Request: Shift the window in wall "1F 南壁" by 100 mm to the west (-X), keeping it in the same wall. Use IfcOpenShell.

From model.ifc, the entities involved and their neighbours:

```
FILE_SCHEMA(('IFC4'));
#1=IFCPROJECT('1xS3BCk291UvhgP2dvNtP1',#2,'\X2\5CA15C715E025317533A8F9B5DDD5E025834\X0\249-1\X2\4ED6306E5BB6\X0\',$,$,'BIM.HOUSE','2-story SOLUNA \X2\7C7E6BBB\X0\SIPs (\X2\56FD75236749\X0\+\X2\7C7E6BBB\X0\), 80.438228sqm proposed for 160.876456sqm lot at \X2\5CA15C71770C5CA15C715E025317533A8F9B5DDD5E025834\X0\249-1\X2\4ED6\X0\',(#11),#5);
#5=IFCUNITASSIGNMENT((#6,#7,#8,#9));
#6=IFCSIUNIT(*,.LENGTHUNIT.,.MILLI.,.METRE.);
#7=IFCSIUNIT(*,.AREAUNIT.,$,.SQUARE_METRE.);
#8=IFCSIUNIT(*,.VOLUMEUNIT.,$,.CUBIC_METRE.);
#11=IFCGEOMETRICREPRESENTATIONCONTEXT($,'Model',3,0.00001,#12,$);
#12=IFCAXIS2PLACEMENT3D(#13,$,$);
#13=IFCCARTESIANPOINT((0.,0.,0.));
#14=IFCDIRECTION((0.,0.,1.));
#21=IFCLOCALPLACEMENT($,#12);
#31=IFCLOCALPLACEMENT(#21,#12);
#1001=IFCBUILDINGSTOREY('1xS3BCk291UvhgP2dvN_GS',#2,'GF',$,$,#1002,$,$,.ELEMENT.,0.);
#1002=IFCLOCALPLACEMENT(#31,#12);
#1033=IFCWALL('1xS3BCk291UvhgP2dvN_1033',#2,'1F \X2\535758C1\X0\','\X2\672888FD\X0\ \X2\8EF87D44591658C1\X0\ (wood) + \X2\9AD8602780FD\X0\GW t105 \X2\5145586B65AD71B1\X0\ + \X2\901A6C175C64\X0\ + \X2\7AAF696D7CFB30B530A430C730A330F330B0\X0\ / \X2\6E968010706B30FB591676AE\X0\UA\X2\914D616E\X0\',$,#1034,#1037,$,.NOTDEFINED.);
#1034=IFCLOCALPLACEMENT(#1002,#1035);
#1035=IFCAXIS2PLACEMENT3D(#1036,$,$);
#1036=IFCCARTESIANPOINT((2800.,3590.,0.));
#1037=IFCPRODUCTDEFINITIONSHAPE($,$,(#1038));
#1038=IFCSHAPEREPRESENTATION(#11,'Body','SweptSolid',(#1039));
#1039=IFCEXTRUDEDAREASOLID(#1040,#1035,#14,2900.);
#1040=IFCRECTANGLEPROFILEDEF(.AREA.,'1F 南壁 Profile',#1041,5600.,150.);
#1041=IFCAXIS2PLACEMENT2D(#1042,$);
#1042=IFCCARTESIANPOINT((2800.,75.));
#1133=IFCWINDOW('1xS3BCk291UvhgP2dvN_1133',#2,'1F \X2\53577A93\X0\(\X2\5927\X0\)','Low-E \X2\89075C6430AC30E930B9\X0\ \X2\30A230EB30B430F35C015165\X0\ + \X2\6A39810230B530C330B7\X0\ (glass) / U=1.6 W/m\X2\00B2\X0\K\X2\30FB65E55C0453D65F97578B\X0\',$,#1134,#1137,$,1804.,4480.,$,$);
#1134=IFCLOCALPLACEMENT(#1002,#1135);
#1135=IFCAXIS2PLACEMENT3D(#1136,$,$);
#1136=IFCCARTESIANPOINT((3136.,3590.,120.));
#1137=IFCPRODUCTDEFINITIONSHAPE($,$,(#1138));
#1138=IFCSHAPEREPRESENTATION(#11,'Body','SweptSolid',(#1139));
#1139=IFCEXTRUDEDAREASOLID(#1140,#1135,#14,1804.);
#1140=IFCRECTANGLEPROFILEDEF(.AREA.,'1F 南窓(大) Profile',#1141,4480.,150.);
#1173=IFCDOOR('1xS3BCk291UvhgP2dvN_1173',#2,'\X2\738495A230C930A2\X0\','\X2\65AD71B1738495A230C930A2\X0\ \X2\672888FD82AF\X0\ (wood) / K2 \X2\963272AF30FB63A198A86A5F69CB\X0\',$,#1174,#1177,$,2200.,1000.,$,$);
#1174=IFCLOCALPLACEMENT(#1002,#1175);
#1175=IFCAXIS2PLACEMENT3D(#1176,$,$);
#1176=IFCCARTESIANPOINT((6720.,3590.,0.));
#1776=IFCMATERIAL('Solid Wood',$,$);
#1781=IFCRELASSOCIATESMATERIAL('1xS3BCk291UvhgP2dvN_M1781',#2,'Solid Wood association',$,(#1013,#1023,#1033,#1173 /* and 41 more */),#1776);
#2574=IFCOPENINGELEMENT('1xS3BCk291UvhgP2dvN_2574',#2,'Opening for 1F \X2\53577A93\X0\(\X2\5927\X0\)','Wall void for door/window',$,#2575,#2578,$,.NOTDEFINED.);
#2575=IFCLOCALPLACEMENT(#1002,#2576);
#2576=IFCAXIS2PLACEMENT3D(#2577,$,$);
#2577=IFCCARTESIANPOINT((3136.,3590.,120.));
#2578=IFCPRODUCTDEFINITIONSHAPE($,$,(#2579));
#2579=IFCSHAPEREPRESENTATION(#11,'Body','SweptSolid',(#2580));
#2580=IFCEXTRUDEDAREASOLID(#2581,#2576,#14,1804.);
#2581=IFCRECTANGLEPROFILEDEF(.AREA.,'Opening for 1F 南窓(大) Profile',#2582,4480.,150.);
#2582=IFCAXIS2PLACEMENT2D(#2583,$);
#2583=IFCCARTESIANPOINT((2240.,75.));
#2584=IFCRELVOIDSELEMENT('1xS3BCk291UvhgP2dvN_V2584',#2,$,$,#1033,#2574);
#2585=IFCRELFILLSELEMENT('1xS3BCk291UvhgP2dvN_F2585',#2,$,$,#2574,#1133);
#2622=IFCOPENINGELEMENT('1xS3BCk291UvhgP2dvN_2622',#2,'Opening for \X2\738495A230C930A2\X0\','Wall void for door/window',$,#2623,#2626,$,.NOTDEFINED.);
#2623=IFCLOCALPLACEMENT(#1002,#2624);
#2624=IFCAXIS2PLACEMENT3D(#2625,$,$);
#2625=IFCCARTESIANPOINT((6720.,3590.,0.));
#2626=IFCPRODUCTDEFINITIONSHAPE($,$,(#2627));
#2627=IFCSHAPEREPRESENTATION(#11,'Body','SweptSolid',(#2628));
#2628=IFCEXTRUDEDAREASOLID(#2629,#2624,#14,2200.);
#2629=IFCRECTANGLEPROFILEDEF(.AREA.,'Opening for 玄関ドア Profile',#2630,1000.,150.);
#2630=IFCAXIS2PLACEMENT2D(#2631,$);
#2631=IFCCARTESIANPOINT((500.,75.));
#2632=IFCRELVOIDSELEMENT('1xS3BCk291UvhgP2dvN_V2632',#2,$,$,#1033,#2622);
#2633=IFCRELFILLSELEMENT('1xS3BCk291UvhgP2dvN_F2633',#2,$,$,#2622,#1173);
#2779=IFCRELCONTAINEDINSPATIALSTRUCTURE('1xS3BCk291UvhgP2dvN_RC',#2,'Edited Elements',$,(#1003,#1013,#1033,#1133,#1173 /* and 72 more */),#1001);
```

```python
import ifcopenshell
import ifcopenshell.api.geometry
import ifcopenshell.util.placement

model = ifcopenshell.open("model.ifc")

window = model.by_guid("1xS3BCk291UvhgP2dvN_1133")
opening = window.FillsVoids[0].RelatingOpeningElement
wall = opening.VoidsElements[0].RelatingBuildingElement

wall_matrix = ifcopenshell.util.placement.get_local_placement(wall.ObjectPlacement)
shift = wall_matrix[:3, 0] * -100.0
before = ifcopenshell.util.placement.get_local_placement(window.ObjectPlacement)[:3, 3].copy()

# The window is not placed relative to its opening, so move both.
for product in (opening, window):
    matrix = ifcopenshell.util.placement.get_local_placement(product.ObjectPlacement)
    matrix[:3, 3] += shift
    ifcopenshell.api.geometry.edit_object_placement(model, product=product, matrix=matrix, is_si=False)

after = ifcopenshell.util.placement.get_local_placement(window.ObjectPlacement)[:3, 3]
print("window moved by", (after - before).round(3) + 0.0)

model.write("model_edited.ifc")
```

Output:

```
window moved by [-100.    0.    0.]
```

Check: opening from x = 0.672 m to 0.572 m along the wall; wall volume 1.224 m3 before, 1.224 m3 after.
